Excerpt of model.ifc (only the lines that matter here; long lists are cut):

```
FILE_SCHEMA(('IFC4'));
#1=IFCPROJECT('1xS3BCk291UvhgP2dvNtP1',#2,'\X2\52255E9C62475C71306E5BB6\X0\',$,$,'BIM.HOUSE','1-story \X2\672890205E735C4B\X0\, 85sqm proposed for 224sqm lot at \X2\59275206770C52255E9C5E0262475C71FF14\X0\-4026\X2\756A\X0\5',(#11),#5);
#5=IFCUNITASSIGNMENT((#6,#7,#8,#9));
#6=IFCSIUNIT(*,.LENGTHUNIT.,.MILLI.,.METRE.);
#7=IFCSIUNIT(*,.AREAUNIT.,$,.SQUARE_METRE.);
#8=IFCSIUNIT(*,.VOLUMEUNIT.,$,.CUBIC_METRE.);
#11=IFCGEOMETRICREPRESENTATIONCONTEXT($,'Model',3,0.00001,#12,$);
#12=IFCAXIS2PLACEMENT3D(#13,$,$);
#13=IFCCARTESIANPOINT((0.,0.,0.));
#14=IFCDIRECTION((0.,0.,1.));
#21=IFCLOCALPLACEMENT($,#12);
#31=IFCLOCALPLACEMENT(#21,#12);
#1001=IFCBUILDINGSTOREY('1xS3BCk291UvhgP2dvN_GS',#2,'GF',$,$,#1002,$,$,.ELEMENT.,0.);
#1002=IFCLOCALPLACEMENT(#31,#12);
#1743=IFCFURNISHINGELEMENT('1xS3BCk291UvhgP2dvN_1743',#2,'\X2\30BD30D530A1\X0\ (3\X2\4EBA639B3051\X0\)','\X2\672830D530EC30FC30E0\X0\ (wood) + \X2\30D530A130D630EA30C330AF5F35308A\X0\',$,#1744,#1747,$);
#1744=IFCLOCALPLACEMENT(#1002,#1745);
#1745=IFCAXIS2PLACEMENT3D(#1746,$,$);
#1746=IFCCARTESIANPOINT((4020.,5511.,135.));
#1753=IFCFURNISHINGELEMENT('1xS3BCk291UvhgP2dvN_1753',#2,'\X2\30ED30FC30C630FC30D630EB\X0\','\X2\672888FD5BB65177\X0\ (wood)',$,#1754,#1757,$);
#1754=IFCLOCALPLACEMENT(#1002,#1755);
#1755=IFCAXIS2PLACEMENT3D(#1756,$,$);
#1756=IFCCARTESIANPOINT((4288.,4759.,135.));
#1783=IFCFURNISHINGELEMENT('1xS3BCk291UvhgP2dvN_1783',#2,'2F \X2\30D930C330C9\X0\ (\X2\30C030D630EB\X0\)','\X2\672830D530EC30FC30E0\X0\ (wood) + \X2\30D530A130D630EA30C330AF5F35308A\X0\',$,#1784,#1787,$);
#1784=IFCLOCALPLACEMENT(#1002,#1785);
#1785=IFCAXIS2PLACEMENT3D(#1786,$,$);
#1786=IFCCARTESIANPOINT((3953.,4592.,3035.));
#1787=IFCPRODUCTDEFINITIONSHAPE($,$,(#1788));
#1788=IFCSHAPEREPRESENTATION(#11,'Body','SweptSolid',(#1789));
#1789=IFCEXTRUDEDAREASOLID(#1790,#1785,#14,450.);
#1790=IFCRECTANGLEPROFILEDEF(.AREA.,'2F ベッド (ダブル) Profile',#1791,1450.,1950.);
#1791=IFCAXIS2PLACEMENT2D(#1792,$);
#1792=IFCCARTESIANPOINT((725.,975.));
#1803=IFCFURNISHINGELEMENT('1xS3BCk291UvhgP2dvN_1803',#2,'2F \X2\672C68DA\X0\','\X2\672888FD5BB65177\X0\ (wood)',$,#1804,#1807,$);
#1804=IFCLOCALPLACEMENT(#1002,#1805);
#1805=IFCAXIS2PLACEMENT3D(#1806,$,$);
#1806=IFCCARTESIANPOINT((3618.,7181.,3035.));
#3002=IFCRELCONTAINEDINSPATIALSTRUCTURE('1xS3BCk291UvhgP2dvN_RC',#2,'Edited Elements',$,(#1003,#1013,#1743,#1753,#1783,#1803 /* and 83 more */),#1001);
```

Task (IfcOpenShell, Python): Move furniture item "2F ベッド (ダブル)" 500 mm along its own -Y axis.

```python
import ifcopenshell
import ifcopenshell.api.geometry
import ifcopenshell.util.placement
import ifcopenshell.util.unit

model = ifcopenshell.open("model.ifc")
unit_scale = ifcopenshell.util.unit.calculate_unit_scale(model)

item = model.by_id(1783)
matrix = ifcopenshell.util.placement.get_local_placement(item.ObjectPlacement)
matrix[:3, 3] -= matrix[:3, 1] * 0.5 / unit_scale
ifcopenshell.api.geometry.edit_object_placement(model, product=item, matrix=matrix, is_si=False)

print(ifcopenshell.util.placement.get_local_placement(item.ObjectPlacement).round(3) + 0.0)

model.write("model_updated.ifc")
```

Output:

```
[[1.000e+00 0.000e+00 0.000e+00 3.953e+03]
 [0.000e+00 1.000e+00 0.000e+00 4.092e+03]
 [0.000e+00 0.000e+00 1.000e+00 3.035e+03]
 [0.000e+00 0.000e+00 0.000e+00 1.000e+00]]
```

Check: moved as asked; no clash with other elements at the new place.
